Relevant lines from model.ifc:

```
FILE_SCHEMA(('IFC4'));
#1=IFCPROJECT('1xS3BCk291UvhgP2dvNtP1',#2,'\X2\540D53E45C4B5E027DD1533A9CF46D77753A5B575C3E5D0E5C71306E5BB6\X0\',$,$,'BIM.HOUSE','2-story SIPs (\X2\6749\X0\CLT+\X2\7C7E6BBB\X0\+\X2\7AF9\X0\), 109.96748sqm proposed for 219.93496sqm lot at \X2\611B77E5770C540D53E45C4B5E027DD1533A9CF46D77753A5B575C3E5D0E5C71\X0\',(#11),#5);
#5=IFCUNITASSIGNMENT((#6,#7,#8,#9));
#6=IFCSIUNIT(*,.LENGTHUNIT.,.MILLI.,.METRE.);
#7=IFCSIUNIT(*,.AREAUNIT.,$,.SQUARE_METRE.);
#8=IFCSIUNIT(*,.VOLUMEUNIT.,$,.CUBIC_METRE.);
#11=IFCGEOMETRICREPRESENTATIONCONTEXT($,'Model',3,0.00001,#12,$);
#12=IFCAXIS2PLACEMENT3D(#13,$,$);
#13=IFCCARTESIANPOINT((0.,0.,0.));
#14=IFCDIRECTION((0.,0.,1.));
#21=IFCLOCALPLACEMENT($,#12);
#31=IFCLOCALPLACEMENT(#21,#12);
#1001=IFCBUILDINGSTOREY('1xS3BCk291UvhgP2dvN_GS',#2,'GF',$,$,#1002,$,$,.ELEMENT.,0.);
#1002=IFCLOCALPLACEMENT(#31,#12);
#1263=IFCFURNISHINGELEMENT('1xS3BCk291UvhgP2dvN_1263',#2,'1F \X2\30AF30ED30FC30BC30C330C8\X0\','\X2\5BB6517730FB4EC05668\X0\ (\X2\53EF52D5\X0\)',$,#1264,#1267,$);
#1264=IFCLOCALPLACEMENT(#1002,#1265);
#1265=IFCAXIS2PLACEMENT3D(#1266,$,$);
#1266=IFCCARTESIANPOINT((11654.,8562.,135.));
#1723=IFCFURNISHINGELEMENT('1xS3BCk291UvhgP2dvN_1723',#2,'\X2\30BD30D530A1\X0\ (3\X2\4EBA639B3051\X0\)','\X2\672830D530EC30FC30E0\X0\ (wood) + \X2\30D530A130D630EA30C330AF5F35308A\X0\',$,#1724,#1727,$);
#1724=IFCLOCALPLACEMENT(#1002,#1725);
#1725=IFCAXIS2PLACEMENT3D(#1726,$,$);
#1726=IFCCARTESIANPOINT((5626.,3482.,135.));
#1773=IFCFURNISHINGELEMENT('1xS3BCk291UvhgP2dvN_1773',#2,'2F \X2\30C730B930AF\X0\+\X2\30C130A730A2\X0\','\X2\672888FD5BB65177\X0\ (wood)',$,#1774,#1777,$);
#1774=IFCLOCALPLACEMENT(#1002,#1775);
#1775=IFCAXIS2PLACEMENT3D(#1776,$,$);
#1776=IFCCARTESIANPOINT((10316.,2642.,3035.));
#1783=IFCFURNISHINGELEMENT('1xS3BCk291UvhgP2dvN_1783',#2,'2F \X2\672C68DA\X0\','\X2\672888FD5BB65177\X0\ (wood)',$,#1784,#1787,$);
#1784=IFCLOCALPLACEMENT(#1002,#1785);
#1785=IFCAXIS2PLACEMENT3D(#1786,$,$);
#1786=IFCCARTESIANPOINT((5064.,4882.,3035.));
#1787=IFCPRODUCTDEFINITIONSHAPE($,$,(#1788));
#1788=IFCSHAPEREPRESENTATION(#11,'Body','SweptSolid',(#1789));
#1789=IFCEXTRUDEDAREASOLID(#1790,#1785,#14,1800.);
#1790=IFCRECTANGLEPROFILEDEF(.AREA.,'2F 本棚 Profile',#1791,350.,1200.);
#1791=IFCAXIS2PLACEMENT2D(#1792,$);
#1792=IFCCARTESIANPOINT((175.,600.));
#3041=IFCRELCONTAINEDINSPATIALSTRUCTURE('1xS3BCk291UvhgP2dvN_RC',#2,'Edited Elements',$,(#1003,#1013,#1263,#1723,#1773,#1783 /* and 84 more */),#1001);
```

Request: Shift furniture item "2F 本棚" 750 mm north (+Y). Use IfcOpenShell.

```python
import ifcopenshell
import ifcopenshell.api.geometry
import ifcopenshell.util.placement

model = ifcopenshell.open("model.ifc")

item = model.by_guid("1xS3BCk291UvhgP2dvN_1783")
matrix = ifcopenshell.util.placement.get_local_placement(item.ObjectPlacement)
matrix[1, 3] += 750.0
ifcopenshell.api.geometry.edit_object_placement(model, product=item, matrix=matrix, is_si=False)

print(ifcopenshell.util.placement.get_local_placement(item.ObjectPlacement).round(3) + 0.0)

model.write("model_edited.ifc")
```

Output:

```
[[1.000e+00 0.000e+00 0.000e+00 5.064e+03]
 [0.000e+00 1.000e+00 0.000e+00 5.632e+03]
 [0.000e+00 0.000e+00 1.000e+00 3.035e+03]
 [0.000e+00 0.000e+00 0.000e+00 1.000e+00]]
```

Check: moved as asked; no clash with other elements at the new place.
